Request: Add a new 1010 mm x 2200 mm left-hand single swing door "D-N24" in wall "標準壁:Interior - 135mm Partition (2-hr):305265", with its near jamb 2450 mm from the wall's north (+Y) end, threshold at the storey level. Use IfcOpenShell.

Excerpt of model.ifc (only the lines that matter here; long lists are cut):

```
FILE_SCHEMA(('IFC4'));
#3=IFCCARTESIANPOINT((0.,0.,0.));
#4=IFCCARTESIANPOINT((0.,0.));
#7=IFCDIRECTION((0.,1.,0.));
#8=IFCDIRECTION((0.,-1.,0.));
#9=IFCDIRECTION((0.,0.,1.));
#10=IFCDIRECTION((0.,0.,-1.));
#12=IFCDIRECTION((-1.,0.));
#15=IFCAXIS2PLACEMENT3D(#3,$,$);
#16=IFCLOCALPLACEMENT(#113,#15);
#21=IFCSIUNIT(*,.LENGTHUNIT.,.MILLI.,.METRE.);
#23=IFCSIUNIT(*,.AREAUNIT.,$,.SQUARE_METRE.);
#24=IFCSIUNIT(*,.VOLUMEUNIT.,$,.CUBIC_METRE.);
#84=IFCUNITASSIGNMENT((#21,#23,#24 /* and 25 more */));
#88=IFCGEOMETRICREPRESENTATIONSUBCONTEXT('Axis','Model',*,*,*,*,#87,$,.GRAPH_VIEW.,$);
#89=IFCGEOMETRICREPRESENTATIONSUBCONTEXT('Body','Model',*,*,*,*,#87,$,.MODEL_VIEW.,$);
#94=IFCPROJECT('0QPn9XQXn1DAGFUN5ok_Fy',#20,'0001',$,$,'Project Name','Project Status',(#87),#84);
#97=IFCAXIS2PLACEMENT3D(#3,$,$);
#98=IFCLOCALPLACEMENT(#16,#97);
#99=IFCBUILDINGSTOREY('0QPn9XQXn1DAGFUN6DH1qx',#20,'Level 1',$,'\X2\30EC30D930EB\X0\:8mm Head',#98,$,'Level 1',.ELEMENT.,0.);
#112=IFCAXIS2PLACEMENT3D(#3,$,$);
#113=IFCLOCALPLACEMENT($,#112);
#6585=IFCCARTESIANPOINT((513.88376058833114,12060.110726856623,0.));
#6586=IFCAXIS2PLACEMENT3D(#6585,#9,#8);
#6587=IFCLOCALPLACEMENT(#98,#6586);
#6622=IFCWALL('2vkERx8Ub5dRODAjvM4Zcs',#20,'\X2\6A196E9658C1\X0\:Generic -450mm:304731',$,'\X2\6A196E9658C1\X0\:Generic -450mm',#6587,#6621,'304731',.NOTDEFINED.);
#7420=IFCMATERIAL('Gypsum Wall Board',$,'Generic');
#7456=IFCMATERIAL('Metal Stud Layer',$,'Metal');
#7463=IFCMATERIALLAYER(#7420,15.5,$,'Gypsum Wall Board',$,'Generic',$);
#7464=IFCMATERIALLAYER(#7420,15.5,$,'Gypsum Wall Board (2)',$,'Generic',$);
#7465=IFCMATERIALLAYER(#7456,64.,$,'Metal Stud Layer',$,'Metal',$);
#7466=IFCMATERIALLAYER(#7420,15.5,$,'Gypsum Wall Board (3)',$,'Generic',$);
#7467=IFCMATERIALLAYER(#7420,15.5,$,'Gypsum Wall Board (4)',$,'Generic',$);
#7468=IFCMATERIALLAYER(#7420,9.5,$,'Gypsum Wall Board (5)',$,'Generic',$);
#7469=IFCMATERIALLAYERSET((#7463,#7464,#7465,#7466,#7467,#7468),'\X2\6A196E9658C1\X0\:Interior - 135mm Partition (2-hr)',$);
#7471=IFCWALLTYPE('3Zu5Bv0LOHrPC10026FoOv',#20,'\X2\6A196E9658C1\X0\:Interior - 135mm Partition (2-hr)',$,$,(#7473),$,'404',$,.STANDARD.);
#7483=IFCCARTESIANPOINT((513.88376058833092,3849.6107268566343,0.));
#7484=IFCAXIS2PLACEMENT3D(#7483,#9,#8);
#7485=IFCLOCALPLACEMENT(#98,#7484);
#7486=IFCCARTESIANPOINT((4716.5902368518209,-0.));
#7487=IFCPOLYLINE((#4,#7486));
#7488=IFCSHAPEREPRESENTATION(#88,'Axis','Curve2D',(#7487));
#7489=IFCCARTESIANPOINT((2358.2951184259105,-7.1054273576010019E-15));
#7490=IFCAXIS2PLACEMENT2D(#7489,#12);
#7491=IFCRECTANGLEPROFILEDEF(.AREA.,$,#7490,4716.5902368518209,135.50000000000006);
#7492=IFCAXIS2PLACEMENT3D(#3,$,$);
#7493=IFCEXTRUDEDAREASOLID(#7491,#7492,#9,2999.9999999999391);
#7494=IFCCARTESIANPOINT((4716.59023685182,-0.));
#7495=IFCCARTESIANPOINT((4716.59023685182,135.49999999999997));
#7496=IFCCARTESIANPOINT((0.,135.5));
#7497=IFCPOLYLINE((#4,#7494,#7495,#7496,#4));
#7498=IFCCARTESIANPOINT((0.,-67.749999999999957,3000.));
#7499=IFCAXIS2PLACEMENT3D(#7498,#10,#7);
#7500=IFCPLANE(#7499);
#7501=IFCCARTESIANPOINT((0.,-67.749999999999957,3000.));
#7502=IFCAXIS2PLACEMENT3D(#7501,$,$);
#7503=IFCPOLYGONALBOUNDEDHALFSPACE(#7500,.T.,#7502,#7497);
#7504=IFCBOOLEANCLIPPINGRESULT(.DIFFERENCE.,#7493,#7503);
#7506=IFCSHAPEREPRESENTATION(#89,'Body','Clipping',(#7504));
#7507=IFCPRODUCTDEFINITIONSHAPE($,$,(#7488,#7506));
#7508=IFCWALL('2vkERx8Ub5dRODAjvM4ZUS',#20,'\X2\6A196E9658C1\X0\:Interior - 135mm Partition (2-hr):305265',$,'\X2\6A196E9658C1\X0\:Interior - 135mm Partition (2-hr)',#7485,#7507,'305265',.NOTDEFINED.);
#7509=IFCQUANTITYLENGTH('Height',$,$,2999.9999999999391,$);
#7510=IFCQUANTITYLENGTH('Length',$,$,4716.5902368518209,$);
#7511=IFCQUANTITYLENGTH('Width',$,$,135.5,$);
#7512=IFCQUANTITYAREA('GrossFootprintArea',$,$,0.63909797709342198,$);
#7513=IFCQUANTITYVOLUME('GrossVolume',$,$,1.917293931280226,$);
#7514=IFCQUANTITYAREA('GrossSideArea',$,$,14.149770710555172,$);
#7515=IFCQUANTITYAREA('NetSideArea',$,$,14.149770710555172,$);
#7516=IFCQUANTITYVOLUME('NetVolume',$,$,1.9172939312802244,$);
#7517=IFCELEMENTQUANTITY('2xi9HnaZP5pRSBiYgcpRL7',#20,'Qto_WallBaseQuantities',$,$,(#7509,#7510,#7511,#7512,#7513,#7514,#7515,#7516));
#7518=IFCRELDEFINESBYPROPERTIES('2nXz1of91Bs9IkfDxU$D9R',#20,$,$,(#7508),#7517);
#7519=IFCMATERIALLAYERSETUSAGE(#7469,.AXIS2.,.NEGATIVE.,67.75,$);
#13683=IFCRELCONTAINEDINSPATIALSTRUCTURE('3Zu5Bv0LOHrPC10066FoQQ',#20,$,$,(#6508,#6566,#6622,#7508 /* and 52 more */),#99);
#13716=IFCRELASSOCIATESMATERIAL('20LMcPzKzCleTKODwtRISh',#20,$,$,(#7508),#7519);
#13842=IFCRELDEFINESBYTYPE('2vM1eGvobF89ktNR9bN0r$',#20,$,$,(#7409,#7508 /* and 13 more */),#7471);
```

```python
import numpy as np
import ifcopenshell
import ifcopenshell.api.feature
import ifcopenshell.api.geometry
import ifcopenshell.api.pset
import ifcopenshell.api.root
import ifcopenshell.api.spatial
import ifcopenshell.geom
import ifcopenshell.util.element
import ifcopenshell.util.placement
import ifcopenshell.util.representation
import ifcopenshell.util.shape
import ifcopenshell.util.unit

model = ifcopenshell.open("model.ifc")
unit_scale = ifcopenshell.util.unit.calculate_unit_scale(model)
area_scale = ifcopenshell.util.unit.calculate_unit_scale(model, "AREAUNIT")
volume_scale = ifcopenshell.util.unit.calculate_unit_scale(model, "VOLUMEUNIT")
settings = ifcopenshell.geom.settings()


def volume(element):
    """Net volume in cubic metres, openings subtracted."""
    shape = ifcopenshell.geom.create_shape(settings, element)
    return ifcopenshell.util.shape.get_volume(shape.geometry)


wall = model.by_guid("2vkERx8Ub5dRODAjvM4ZUS")
storey = ifcopenshell.util.element.get_container(wall, ifc_class="IfcBuildingStorey")
context = ifcopenshell.util.representation.get_context(model, "Model", "Body", "MODEL_VIEW")
before = volume(wall)

width, height, from_end, sill = 1.01, 2.2, 2.45, 0.0  # metres

# The wall runs along its own X axis, and the end named is its -X end.
wall_shape = ifcopenshell.geom.create_shape(settings, wall)
x, y, z = ifcopenshell.util.shape.get_vertices(wall_shape.geometry).T
start = x.min() + from_end
face, thickness = float(y.min()), float(y.max() - y.min())
wall_matrix = ifcopenshell.util.placement.get_local_placement(wall.ObjectPlacement)
level = ifcopenshell.util.placement.get_local_placement(storey.ObjectPlacement)[2, 3]


def in_wall(x, y):
    """Placement at x, y metres in the wall's axes, at sill height."""
    matrix = wall_matrix.copy()
    matrix[:, 3] = wall_matrix @ np.array([x / unit_scale, y / unit_scale, 0.0, 1.0])
    matrix[2, 3] = level + sill / unit_scale
    return matrix


# Opening: a box that overshoots both wall faces by 50 mm.
opening = ifcopenshell.api.root.create_entity(model, ifc_class="IfcOpeningElement", predefined_type="OPENING")
box = ifcopenshell.api.geometry.add_wall_representation(
    model, context=context, length=width, height=height, thickness=thickness + 0.1
)
ifcopenshell.api.geometry.assign_representation(model, product=opening, representation=box)
ifcopenshell.api.geometry.edit_object_placement(model, product=opening, matrix=in_wall(start, face - 0.05), is_si=False)
ifcopenshell.api.feature.add_feature(model, feature=opening, element=wall)

door = ifcopenshell.api.root.create_entity(model, ifc_class="IfcDoor", name="D-N24", predefined_type="DOOR")
door.OverallWidth, door.OverallHeight = width / unit_scale, height / unit_scale
door.OperationType = "SINGLE_SWING_LEFT"
body = ifcopenshell.api.geometry.add_door_representation(
    model,
    context=context,
    overall_width=door.OverallWidth,
    overall_height=door.OverallHeight,
    operation_type="SINGLE_SWING_LEFT",
    lining_properties={"LiningDepth": thickness / unit_scale, "ThresholdDepth": thickness / unit_scale},
)
ifcopenshell.api.geometry.assign_representation(model, product=door, representation=body)
ifcopenshell.api.spatial.assign_container(model, products=[door], relating_structure=storey)
ifcopenshell.api.feature.add_filling(model, opening=opening, element=door)

# The lining spans the wall, so the door starts at the wall face.
ifcopenshell.api.geometry.edit_object_placement(model, product=door, matrix=in_wall(start, face), is_si=False)

after = volume(wall)

# Update the wall's stored quantities.
qto = model.by_id(ifcopenshell.util.element.get_pset(wall, "Qto_WallBaseQuantities", should_inherit=False)["id"])
ifcopenshell.api.pset.edit_qto(model, qto=qto, properties={
    "NetSideArea": after / thickness / area_scale,
    "NetVolume": after / volume_scale,
})

print(f"wall volume {before:.3f} -> {after:.3f} m3")

model.write("model_v2.ifc")
```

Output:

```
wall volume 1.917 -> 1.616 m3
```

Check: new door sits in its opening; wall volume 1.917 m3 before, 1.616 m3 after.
